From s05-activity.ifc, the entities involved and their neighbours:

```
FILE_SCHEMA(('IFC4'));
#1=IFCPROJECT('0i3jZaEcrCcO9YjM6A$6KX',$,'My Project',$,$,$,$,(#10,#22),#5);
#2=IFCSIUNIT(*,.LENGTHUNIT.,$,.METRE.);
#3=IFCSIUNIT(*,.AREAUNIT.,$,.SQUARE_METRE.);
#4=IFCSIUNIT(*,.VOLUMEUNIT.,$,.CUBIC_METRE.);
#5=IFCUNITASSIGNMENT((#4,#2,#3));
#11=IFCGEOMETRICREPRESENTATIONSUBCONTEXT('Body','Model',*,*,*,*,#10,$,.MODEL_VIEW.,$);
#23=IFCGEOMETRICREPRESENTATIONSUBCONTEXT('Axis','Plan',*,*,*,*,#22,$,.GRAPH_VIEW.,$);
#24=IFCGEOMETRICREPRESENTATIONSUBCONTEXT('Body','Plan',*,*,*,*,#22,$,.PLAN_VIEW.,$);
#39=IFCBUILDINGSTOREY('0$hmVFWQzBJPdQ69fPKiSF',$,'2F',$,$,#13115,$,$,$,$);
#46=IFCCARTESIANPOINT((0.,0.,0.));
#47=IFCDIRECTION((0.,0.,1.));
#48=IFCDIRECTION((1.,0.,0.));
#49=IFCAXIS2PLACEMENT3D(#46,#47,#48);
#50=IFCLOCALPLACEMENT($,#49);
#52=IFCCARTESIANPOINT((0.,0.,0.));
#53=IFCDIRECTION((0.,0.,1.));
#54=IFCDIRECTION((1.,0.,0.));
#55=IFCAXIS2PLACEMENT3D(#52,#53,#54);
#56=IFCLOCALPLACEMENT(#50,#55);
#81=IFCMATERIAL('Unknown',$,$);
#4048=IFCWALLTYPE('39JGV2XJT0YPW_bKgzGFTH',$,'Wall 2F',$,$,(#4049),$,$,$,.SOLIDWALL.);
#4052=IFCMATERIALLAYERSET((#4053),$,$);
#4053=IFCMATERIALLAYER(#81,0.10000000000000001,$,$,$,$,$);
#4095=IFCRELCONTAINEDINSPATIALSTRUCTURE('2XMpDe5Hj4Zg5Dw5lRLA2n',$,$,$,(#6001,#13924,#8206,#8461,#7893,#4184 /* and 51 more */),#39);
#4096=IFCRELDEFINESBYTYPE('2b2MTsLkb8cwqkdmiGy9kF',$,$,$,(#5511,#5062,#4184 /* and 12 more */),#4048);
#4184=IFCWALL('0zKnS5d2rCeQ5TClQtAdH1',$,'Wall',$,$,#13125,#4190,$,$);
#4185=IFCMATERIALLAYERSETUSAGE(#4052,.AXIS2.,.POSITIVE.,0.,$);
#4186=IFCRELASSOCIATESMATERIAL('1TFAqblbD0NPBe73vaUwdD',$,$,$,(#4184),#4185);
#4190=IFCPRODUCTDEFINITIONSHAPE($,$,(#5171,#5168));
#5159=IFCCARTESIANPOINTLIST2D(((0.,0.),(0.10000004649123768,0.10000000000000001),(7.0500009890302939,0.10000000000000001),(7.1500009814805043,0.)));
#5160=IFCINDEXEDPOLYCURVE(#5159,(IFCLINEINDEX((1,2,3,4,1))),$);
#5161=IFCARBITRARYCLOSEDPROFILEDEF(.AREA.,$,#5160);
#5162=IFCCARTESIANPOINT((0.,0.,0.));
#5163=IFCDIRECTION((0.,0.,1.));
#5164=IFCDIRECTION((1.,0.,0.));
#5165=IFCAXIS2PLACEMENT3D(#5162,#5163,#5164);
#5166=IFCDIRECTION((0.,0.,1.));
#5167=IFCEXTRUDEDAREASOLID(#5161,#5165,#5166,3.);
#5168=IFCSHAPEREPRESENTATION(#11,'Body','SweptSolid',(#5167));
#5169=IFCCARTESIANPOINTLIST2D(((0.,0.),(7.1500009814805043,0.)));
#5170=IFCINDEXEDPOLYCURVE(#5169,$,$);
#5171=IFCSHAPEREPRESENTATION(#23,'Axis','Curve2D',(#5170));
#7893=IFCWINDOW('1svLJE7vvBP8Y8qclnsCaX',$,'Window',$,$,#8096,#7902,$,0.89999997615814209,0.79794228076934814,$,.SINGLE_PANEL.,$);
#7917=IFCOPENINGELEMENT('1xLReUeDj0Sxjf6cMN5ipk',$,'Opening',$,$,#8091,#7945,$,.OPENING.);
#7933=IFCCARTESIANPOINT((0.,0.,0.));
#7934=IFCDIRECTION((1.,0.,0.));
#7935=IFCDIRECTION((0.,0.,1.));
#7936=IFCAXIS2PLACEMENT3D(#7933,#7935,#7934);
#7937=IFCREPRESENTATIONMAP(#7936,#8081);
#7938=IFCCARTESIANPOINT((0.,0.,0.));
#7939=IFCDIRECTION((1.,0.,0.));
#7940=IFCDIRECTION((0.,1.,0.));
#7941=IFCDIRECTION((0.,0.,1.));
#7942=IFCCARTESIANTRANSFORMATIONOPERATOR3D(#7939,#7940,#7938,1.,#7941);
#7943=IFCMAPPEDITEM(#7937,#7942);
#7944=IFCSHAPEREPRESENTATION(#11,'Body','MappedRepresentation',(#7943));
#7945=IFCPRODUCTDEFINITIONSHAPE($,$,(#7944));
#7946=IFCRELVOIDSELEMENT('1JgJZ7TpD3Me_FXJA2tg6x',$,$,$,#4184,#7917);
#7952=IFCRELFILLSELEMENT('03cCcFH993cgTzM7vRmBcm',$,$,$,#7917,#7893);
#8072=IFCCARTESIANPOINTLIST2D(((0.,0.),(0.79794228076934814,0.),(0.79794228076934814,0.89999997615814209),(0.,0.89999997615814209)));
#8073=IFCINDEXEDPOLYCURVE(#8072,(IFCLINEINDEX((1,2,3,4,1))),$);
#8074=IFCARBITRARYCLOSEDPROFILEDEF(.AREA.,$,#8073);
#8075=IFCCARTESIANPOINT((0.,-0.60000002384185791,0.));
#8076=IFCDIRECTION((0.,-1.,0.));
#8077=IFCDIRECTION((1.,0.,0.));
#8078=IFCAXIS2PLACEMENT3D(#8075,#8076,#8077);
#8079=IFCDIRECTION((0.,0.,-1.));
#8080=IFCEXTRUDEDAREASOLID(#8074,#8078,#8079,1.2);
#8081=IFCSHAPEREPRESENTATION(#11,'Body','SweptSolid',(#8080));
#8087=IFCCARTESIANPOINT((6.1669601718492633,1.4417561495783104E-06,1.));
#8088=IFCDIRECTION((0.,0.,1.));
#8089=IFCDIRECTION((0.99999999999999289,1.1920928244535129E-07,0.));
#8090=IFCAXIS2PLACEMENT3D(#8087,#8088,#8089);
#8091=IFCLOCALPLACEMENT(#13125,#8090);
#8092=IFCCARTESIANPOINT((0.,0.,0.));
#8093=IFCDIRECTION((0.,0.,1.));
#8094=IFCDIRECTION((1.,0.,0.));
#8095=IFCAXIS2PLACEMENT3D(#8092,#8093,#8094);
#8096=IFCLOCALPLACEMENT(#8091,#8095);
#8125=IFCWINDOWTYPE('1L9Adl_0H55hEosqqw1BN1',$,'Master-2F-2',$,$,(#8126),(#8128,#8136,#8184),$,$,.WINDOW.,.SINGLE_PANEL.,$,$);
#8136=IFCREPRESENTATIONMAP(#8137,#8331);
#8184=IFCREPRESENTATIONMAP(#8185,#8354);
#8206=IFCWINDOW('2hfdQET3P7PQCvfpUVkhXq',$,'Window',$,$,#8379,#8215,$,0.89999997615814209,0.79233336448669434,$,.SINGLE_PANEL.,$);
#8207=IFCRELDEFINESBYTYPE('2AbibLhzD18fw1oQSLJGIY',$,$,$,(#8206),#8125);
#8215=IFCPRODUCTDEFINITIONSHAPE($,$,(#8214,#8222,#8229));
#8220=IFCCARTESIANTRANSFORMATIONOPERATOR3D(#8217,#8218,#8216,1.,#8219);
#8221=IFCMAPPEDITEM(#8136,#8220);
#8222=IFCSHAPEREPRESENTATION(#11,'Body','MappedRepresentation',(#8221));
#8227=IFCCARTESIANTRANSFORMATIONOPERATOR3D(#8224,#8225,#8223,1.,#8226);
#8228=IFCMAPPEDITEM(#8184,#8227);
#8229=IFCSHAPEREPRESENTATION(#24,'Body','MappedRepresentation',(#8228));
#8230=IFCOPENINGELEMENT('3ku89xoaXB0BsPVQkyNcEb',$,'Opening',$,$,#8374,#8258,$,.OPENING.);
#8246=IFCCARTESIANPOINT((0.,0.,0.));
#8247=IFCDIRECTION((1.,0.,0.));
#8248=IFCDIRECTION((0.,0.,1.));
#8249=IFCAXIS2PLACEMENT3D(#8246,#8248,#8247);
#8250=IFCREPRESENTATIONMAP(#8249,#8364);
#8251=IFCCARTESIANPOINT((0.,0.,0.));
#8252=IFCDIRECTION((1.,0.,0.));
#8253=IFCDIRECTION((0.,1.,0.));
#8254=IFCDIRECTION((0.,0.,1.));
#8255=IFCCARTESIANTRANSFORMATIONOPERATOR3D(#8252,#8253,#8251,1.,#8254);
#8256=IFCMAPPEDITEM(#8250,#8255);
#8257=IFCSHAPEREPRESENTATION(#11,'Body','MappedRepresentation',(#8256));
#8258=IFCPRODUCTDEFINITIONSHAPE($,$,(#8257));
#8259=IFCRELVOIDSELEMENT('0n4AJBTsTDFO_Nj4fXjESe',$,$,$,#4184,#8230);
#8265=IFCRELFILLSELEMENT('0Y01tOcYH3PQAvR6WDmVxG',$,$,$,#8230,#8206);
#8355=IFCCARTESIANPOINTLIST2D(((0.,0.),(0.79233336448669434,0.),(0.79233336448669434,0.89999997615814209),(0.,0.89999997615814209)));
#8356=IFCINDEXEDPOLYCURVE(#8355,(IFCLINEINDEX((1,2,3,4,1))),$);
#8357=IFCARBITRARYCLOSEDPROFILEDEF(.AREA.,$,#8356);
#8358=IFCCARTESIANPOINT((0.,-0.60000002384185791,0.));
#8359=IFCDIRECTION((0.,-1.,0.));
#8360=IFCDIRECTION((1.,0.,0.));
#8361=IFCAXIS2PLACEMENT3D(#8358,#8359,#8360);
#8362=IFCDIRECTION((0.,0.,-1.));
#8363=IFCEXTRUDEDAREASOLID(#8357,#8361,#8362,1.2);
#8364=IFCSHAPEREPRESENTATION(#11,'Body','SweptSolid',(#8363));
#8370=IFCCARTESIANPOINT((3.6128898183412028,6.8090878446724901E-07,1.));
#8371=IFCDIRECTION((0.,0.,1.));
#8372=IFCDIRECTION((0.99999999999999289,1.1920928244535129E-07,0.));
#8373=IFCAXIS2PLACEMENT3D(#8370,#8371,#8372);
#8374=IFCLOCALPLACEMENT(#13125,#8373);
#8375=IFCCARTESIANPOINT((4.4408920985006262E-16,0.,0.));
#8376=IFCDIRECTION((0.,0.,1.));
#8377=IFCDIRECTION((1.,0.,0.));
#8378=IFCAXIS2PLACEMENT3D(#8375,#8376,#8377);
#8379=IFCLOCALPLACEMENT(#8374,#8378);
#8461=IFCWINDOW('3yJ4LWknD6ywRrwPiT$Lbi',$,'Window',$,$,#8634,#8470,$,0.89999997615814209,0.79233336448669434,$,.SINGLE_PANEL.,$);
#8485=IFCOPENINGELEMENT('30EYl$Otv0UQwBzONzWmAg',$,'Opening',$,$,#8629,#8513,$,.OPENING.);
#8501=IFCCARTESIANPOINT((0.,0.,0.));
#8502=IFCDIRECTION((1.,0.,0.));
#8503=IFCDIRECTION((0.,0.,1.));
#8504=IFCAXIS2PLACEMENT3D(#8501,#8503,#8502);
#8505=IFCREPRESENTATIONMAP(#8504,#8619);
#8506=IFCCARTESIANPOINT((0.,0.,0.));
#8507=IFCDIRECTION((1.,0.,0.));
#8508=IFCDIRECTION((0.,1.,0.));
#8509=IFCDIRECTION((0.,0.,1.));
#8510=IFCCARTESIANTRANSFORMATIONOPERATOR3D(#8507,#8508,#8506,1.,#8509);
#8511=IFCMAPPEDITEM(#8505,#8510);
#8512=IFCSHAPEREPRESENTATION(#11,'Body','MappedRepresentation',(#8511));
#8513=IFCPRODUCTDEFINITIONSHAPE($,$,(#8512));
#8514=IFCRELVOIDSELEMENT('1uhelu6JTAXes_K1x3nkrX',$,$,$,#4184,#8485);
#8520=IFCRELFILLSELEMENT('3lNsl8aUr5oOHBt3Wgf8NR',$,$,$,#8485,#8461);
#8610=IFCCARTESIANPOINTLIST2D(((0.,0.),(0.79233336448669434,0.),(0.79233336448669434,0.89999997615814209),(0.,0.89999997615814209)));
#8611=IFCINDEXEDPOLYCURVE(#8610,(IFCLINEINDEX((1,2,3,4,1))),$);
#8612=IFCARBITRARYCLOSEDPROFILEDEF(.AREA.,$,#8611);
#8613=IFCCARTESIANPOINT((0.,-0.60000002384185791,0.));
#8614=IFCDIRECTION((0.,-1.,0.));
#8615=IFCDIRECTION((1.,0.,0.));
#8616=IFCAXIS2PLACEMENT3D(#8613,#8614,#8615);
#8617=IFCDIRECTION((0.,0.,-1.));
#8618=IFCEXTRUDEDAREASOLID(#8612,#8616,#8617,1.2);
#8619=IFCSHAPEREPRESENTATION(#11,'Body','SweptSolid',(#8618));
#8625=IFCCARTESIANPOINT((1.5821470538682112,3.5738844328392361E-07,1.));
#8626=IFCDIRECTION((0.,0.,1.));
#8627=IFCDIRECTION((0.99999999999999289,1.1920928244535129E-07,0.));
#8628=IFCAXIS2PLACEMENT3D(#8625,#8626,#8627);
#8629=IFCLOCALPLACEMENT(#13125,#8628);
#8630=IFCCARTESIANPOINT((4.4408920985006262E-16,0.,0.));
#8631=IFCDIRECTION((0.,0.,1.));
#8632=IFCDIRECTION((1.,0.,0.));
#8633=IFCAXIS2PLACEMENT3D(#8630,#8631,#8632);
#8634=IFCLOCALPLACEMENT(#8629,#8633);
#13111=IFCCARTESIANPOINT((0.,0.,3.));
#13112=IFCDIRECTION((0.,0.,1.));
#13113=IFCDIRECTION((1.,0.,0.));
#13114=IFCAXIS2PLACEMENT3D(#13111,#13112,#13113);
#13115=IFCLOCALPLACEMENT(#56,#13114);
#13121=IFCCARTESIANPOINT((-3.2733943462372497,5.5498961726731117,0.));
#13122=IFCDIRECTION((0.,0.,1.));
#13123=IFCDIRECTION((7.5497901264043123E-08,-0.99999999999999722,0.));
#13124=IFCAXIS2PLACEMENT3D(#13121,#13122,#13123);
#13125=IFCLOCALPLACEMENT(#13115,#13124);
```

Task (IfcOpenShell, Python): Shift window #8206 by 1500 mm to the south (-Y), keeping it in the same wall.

```python
import ifcopenshell
import ifcopenshell.api.geometry
import ifcopenshell.util.placement

model = ifcopenshell.open("s05-activity.ifc")

window = model.by_guid("2hfdQET3P7PQCvfpUVkhXq")
opening = window.FillsVoids[0].RelatingOpeningElement
wall = opening.VoidsElements[0].RelatingBuildingElement

wall_matrix = ifcopenshell.util.placement.get_local_placement(wall.ObjectPlacement)
shift = wall_matrix[:3, 0] * 1.5
before = ifcopenshell.util.placement.get_local_placement(window.ObjectPlacement)[:3, 3].copy()

# The window is placed relative to its opening, so it follows when the opening moves.
matrix = ifcopenshell.util.placement.get_local_placement(opening.ObjectPlacement)
matrix[:3, 3] += shift
ifcopenshell.api.geometry.edit_object_placement(
    model, product=opening, matrix=matrix, is_si=False, should_transform_children=True
)

after = ifcopenshell.util.placement.get_local_placement(window.ObjectPlacement)[:3, 3]
print("window moved by", (after - before).round(3) + 0.0)

model.write("s05-activity_v2.ifc")
```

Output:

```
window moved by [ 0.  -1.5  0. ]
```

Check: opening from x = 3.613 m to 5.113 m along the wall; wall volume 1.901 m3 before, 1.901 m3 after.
